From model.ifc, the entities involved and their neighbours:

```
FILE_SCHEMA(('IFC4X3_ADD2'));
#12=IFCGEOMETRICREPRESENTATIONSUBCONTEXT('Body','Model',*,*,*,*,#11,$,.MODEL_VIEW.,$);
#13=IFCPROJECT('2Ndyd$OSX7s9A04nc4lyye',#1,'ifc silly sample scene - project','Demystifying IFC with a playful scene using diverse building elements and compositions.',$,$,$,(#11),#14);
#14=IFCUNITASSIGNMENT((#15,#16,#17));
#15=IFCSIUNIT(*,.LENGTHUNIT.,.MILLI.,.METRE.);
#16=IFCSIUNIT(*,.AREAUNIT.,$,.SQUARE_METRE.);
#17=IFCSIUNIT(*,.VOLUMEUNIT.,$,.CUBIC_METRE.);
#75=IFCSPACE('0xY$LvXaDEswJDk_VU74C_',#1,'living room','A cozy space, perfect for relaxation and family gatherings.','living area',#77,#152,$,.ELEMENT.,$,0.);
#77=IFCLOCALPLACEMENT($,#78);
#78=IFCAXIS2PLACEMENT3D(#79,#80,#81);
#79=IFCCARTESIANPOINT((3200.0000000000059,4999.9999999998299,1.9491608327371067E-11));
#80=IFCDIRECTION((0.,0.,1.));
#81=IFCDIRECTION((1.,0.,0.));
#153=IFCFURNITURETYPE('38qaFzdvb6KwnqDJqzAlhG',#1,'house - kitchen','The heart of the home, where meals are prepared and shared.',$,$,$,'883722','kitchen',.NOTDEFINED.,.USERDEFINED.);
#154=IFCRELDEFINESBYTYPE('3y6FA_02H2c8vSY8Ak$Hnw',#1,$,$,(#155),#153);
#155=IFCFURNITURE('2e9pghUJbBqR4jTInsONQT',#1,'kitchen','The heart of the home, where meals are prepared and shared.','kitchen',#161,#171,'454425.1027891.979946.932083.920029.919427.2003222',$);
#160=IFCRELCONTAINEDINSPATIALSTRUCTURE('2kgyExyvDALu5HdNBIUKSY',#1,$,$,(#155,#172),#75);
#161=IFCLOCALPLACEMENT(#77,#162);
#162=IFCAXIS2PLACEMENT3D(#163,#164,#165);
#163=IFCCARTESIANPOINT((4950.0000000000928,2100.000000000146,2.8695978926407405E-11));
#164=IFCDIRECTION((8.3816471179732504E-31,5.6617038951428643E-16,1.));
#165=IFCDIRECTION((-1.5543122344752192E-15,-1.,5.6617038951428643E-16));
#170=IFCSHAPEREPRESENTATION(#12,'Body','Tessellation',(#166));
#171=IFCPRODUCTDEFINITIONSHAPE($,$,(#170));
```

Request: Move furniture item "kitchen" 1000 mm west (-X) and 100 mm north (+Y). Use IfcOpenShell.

```python
import ifcopenshell
import ifcopenshell.api.geometry
import ifcopenshell.util.placement

model = ifcopenshell.open("model.ifc")

item = model.by_guid("2e9pghUJbBqR4jTInsONQT")
matrix = ifcopenshell.util.placement.get_local_placement(item.ObjectPlacement)
matrix[0, 3] -= 1000.0
matrix[1, 3] += 100.0
ifcopenshell.api.geometry.edit_object_placement(model, product=item, matrix=matrix, is_si=False)

print(ifcopenshell.util.placement.get_local_placement(item.ObjectPlacement).round(3) + 0.0)

model.write("model_v2.ifc")
```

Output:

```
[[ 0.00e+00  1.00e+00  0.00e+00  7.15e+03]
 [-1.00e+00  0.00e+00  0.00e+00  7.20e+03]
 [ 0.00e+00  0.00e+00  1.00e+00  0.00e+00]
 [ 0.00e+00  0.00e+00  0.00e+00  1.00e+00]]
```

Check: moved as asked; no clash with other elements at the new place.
